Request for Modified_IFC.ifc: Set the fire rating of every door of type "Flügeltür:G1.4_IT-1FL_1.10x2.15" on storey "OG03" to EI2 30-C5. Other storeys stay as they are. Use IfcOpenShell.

First a look at what the model holds.

```python
import ifcopenshell
import ifcopenshell.util.element

model = ifcopenshell.open("Modified_IFC.ifc")
print(model.schema)
storey = next(s for s in model.by_type("IfcBuildingStorey") if s.Name == "OG03")
doors = [e for e in ifcopenshell.util.element.get_decomposition(storey) if e.is_a("IfcDoor")]
seen = {}
for e in doors:
    element_type = ifcopenshell.util.element.get_type(e)
    key = (element_type.Name if element_type != e and element_type else None, ifcopenshell.util.element.get_pset(e, "Pset_DoorCommon", "FireRating"))
    seen[key] = seen.get(key, 0) + 1
for (name, value), count in sorted(seen.items(), key=str):
    print(count, "x", name, "|", value)
```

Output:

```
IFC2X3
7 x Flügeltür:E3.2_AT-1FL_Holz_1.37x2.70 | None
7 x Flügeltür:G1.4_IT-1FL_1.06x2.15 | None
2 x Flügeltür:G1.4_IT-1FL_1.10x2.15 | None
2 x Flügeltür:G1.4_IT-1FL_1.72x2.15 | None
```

```python
import ifcopenshell
import ifcopenshell.api.pset
import ifcopenshell.util.element

model = ifcopenshell.open("Modified_IFC.ifc")

storey = next(s for s in model.by_type("IfcBuildingStorey") if s.Name == "OG03")
doors = [e for e in ifcopenshell.util.element.get_decomposition(storey) if e.is_a("IfcDoor")]

count = 0
for e in doors:
    element_type = ifcopenshell.util.element.get_type(e)
    if element_type in (None, e) or element_type.Name != "Flügeltür:G1.4_IT-1FL_1.10x2.15":
        continue
    # add_pset returns the element's existing set when there is one.
    pset = ifcopenshell.api.pset.add_pset(model, product=e, name="Pset_DoorCommon")
    ifcopenshell.api.pset.edit_pset(model, pset=pset, properties={"FireRating": "EI2 30-C5"})
    count += 1

print(count, "doors updated")

model.write("Modified_IFC_v2.ifc")
```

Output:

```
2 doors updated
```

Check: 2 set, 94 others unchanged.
